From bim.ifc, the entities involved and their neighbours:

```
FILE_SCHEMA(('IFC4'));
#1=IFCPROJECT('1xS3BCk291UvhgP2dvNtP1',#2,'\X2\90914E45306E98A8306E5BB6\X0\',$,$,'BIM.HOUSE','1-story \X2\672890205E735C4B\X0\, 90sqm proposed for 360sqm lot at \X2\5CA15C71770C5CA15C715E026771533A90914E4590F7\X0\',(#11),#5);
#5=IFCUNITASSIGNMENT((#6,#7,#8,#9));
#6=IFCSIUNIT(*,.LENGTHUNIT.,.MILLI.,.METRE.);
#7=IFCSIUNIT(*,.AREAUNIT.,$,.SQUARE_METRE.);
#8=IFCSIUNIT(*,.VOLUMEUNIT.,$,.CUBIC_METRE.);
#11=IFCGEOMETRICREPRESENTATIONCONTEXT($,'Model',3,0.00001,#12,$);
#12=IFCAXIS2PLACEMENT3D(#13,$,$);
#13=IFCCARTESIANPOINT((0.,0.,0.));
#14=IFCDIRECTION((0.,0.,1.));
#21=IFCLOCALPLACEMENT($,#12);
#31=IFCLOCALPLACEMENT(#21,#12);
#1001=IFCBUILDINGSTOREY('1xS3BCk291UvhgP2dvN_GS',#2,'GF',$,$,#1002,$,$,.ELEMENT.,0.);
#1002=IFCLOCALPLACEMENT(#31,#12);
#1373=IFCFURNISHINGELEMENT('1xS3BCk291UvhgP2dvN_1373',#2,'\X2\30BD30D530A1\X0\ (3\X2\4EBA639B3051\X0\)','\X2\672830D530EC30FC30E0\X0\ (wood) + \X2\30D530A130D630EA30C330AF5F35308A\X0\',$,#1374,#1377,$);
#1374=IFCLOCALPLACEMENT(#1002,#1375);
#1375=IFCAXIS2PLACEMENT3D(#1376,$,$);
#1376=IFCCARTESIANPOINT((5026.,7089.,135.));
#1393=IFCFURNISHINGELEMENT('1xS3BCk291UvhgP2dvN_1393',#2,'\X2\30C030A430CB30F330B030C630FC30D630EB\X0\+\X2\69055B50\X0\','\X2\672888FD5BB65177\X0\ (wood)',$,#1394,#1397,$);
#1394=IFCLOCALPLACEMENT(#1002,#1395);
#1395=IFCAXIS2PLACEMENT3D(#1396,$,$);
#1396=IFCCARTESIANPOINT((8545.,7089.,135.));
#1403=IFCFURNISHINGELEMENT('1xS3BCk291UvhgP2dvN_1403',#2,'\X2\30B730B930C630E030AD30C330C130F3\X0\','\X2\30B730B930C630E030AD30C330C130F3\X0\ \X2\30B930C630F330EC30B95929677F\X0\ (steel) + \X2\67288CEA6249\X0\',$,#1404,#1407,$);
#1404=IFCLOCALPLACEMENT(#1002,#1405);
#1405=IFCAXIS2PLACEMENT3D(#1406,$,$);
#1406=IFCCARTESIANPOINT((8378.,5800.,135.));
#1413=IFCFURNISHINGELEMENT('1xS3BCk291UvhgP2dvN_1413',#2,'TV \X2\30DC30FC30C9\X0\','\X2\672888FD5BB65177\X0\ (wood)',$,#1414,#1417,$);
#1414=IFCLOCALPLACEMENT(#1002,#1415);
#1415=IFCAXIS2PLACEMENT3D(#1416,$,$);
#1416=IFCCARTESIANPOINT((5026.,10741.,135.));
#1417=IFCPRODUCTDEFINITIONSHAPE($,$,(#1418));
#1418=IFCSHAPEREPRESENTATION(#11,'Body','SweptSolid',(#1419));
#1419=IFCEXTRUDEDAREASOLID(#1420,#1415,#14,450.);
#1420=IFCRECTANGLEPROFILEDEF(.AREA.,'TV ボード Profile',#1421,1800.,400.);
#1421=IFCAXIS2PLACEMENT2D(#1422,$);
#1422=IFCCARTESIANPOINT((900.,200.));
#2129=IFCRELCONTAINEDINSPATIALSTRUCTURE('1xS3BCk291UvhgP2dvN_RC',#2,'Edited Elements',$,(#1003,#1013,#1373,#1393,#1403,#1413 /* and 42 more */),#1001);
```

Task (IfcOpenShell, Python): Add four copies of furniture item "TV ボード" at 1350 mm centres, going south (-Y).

```python
import numpy as np
import ifcopenshell
import ifcopenshell.api.geometry
import ifcopenshell.api.root
import ifcopenshell.util.element
import ifcopenshell.util.placement

model = ifcopenshell.open("bim.ifc")


def reuse_history(source, copy):
    """copy_class also copies each property set's owner history, people and application; keep the originals."""
    for rel in copy.IsDefinedBy:
        if rel.is_a("IfcRelDefinesByProperties") and (history := rel.RelatingPropertyDefinition.OwnerHistory):
            rel.RelatingPropertyDefinition.OwnerHistory = source.OwnerHistory
            ifcopenshell.util.element.remove_deep2(model, history)


source = model.by_id(1413)
base = ifcopenshell.util.placement.get_local_placement(source.ObjectPlacement)
step = np.array([0.0, -1.0, 0.0]) * 1350.0

for i in range(1, 5):
    copy = ifcopenshell.api.root.copy_class(model, product=source)
    copy.Representation = ifcopenshell.util.element.copy_deep(
        model, source.Representation, exclude=["IfcGeometricRepresentationContext", "IfcRepresentationMap"]
    )
    reuse_history(source, copy)
    matrix = base.copy()
    matrix[:3, 3] += i * step
    print("added at", matrix[:3, 3].round(3) + 0.0)
    ifcopenshell.api.geometry.edit_object_placement(model, product=copy, matrix=matrix, is_si=False)

model.write("bim_updated.ifc")
```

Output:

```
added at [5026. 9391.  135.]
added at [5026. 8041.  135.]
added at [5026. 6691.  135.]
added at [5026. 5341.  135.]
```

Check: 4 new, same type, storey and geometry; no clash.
